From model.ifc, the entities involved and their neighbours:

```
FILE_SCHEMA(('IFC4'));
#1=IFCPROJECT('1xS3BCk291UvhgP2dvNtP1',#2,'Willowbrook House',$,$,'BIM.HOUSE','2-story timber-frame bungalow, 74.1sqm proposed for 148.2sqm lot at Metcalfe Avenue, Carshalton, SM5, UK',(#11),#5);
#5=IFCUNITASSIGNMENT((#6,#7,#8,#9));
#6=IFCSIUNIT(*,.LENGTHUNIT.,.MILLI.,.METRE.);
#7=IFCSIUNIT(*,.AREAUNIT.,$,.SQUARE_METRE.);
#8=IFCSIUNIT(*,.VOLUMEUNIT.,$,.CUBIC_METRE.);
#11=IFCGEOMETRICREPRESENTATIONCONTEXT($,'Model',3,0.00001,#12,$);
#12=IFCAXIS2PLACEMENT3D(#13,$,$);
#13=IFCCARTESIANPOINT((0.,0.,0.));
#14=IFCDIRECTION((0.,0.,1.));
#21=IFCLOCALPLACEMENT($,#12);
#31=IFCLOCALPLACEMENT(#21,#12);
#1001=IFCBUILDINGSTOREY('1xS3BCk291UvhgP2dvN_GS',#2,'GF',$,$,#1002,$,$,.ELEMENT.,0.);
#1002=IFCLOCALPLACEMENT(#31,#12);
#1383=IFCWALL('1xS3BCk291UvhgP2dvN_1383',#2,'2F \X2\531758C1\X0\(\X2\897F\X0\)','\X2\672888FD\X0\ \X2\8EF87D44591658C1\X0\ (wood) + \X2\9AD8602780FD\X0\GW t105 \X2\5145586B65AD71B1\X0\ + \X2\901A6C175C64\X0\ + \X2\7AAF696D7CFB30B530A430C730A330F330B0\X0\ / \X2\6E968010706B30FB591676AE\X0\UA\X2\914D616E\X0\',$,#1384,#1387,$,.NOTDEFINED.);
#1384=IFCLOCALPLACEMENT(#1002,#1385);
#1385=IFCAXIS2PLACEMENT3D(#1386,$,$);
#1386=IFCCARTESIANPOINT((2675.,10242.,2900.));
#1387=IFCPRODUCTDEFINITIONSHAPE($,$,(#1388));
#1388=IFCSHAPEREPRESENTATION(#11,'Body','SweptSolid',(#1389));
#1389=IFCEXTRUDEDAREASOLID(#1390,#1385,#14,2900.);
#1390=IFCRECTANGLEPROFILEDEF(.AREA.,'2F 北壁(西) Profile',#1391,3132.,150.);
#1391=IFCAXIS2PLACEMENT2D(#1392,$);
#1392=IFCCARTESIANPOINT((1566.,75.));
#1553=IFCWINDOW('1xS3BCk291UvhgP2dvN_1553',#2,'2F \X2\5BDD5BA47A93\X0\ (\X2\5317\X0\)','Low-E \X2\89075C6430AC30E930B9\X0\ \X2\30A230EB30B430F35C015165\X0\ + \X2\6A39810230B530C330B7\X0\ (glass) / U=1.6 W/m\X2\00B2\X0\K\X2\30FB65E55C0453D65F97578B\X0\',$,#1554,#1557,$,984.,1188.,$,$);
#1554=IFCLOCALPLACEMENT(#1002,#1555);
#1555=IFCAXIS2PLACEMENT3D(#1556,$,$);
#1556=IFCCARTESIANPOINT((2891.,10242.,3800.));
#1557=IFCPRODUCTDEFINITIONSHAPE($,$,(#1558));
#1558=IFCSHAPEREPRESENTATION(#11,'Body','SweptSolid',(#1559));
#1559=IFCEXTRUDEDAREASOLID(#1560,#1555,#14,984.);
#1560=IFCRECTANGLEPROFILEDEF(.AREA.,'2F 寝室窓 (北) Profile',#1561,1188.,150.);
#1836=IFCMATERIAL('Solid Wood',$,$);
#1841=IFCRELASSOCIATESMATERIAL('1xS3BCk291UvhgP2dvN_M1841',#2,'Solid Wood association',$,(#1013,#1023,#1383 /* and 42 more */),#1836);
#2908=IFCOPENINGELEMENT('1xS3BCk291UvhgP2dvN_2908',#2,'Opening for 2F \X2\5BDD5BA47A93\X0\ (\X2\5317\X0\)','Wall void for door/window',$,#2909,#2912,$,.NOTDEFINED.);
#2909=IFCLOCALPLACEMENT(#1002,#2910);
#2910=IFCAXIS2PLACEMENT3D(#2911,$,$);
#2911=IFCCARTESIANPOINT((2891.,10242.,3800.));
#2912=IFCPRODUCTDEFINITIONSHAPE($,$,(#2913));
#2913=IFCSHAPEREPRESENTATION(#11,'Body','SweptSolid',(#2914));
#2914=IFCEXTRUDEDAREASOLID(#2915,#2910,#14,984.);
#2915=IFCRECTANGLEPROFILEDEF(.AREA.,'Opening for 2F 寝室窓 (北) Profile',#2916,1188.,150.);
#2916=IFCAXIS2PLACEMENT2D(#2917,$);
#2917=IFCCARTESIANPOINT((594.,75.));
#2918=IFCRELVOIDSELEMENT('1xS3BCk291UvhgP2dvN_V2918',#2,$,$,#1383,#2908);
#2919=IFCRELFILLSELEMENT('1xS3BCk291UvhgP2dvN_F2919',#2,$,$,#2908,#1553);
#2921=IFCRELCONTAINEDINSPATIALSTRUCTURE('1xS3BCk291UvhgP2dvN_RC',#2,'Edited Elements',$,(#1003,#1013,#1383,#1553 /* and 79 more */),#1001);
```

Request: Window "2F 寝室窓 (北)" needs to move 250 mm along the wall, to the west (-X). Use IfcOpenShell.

```python
import ifcopenshell
import ifcopenshell.api.geometry
import ifcopenshell.util.placement
import ifcopenshell.util.unit

model = ifcopenshell.open("model.ifc")
unit_scale = ifcopenshell.util.unit.calculate_unit_scale(model)

window = model.by_guid("1xS3BCk291UvhgP2dvN_1553")
opening = window.FillsVoids[0].RelatingOpeningElement
wall = opening.VoidsElements[0].RelatingBuildingElement

wall_matrix = ifcopenshell.util.placement.get_local_placement(wall.ObjectPlacement)
shift = wall_matrix[:3, 0] * -0.25 / unit_scale
before = ifcopenshell.util.placement.get_local_placement(window.ObjectPlacement)[:3, 3].copy()

# The window is not placed relative to its opening, so move both.
for product in (opening, window):
    matrix = ifcopenshell.util.placement.get_local_placement(product.ObjectPlacement)
    matrix[:3, 3] += shift
    ifcopenshell.api.geometry.edit_object_placement(model, product=product, matrix=matrix, is_si=False)

after = ifcopenshell.util.placement.get_local_placement(window.ObjectPlacement)[:3, 3]
print("window moved by", (after - before).round(3) + 0.0)

model.write("model_edited.ifc")
```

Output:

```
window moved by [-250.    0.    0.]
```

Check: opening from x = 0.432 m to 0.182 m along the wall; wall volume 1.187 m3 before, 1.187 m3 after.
